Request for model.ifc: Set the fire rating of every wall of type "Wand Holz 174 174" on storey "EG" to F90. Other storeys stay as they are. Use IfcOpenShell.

First a look at what the model holds.

```python
import ifcopenshell
import ifcopenshell.util.element

model = ifcopenshell.open("model.ifc")
print(model.schema)
storey = next(s for s in model.by_type("IfcBuildingStorey") if s.Name == "EG")
walls = [e for e in ifcopenshell.util.element.get_decomposition(storey) if e.is_a("IfcWall")]
seen = {}
for e in walls:
    element_type = ifcopenshell.util.element.get_type(e)
    key = (element_type.Name if element_type != e and element_type else None, ifcopenshell.util.element.get_pset(e, "Pset_WallCommon", "FireRating"))
    seen[key] = seen.get(key, 0) + 1
for (name, value), count in sorted(seen.items(), key=str):
    print(count, "x", name, "|", value)
```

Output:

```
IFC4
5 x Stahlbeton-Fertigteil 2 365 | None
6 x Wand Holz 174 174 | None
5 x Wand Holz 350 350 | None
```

```python
import ifcopenshell
import ifcopenshell.api.pset
import ifcopenshell.util.element

model = ifcopenshell.open("model.ifc")

storey = next(s for s in model.by_type("IfcBuildingStorey") if s.Name == "EG")
walls = [e for e in ifcopenshell.util.element.get_decomposition(storey) if e.is_a("IfcWall")]

count = 0
for e in walls:
    element_type = ifcopenshell.util.element.get_type(e)
    if element_type in (None, e) or element_type.Name != "Wand Holz 174 174":
        continue
    # add_pset returns the element's existing set when there is one.
    pset = ifcopenshell.api.pset.add_pset(model, product=e, name="Pset_WallCommon")
    ifcopenshell.api.pset.edit_pset(model, pset=pset, properties={"FireRating": "F90"})
    count += 1

print(count, "walls updated")

model.write("model_updated.ifc")
```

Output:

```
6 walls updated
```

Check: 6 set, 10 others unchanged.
